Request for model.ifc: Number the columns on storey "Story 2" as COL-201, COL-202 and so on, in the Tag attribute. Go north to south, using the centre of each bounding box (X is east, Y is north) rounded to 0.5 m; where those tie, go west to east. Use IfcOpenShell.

First a look at what the model holds.

```python
import ifcopenshell
import ifcopenshell.util.element
import ifcopenshell.util.placement

model = ifcopenshell.open("model.ifc")
print(model.schema)
storey = next(s for s in model.by_type("IfcBuildingStorey") if s.Name == "Story 2")
columns = [e for e in ifcopenshell.util.element.get_decomposition(storey) if e.is_a("IfcColumn")]
for e in sorted(columns, key=lambda e: e.id()):
    origin = ifcopenshell.util.placement.get_local_placement(e.ObjectPlacement)[:3, 3]
    print(e.id(), e.Tag, e.Name, origin.round(2) + 0.0, sep=" | ")
```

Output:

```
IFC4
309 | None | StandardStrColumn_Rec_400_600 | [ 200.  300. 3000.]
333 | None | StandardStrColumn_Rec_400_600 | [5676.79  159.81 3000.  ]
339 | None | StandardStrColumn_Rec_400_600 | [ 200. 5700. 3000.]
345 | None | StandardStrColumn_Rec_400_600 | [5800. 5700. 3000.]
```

```python
import ifcopenshell
import ifcopenshell.geom
import ifcopenshell.util.element
import ifcopenshell.util.shape

model = ifcopenshell.open("model.ifc")
settings = ifcopenshell.geom.settings()
settings.set("use-world-coords", True)


def centre(element):
    shape = ifcopenshell.geom.create_shape(settings, element)
    return ifcopenshell.util.shape.get_bbox_centroid(shape.geometry)


storey = next(s for s in model.by_type("IfcBuildingStorey") if s.Name == "Story 2")
columns = [e for e in ifcopenshell.util.element.get_decomposition(storey) if e.is_a("IfcColumn")]

# Insertion points can sit at a corner or the storey origin, so sort by the geometry (in metres).
centres = {e: centre(e) for e in columns}
columns.sort(key=lambda e: (-round(centres[e][1] / 0.5), centres[e][0]))

for i, e in enumerate(columns, start=1):
    number = f"COL-2{i:02d}"
    e.Tag = number
    print(e.id(), number)

model.write("model_edited.ifc")
```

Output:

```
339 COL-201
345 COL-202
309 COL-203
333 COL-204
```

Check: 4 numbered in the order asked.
